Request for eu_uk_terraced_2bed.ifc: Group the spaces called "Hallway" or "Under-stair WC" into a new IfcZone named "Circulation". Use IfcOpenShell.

First a look at what the model holds.

```python
import ifcopenshell

model = ifcopenshell.open("eu_uk_terraced_2bed.ifc")
print(model.schema)
seen = {}
for space in model.by_type("IfcSpace"):
    seen[space.LongName] = seen.get(space.LongName, 0) + 1
for name, count in sorted(seen.items(), key=str):
    print(count, "x", name)
print("zones:", [z.Name for z in model.by_type("IfcZone")][:20])
```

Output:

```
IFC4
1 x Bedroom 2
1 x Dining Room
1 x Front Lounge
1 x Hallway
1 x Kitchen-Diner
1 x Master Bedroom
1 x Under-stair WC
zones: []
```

```python
import ifcopenshell
import ifcopenshell.api.group
import ifcopenshell.api.root

model = ifcopenshell.open("eu_uk_terraced_2bed.ifc")

names = {"Hallway", "Under-stair WC"}
spaces = [s for s in model.by_type("IfcSpace") if s.LongName in names]

zone = ifcopenshell.api.root.create_entity(model, ifc_class="IfcZone", name="Circulation")
ifcopenshell.api.group.assign_group(model, products=spaces, group=zone)
print(len(spaces), "spaces in", zone.Name)

model.write("eu_uk_terraced_2bed_updated.ifc")
```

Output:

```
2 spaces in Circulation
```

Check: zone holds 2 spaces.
